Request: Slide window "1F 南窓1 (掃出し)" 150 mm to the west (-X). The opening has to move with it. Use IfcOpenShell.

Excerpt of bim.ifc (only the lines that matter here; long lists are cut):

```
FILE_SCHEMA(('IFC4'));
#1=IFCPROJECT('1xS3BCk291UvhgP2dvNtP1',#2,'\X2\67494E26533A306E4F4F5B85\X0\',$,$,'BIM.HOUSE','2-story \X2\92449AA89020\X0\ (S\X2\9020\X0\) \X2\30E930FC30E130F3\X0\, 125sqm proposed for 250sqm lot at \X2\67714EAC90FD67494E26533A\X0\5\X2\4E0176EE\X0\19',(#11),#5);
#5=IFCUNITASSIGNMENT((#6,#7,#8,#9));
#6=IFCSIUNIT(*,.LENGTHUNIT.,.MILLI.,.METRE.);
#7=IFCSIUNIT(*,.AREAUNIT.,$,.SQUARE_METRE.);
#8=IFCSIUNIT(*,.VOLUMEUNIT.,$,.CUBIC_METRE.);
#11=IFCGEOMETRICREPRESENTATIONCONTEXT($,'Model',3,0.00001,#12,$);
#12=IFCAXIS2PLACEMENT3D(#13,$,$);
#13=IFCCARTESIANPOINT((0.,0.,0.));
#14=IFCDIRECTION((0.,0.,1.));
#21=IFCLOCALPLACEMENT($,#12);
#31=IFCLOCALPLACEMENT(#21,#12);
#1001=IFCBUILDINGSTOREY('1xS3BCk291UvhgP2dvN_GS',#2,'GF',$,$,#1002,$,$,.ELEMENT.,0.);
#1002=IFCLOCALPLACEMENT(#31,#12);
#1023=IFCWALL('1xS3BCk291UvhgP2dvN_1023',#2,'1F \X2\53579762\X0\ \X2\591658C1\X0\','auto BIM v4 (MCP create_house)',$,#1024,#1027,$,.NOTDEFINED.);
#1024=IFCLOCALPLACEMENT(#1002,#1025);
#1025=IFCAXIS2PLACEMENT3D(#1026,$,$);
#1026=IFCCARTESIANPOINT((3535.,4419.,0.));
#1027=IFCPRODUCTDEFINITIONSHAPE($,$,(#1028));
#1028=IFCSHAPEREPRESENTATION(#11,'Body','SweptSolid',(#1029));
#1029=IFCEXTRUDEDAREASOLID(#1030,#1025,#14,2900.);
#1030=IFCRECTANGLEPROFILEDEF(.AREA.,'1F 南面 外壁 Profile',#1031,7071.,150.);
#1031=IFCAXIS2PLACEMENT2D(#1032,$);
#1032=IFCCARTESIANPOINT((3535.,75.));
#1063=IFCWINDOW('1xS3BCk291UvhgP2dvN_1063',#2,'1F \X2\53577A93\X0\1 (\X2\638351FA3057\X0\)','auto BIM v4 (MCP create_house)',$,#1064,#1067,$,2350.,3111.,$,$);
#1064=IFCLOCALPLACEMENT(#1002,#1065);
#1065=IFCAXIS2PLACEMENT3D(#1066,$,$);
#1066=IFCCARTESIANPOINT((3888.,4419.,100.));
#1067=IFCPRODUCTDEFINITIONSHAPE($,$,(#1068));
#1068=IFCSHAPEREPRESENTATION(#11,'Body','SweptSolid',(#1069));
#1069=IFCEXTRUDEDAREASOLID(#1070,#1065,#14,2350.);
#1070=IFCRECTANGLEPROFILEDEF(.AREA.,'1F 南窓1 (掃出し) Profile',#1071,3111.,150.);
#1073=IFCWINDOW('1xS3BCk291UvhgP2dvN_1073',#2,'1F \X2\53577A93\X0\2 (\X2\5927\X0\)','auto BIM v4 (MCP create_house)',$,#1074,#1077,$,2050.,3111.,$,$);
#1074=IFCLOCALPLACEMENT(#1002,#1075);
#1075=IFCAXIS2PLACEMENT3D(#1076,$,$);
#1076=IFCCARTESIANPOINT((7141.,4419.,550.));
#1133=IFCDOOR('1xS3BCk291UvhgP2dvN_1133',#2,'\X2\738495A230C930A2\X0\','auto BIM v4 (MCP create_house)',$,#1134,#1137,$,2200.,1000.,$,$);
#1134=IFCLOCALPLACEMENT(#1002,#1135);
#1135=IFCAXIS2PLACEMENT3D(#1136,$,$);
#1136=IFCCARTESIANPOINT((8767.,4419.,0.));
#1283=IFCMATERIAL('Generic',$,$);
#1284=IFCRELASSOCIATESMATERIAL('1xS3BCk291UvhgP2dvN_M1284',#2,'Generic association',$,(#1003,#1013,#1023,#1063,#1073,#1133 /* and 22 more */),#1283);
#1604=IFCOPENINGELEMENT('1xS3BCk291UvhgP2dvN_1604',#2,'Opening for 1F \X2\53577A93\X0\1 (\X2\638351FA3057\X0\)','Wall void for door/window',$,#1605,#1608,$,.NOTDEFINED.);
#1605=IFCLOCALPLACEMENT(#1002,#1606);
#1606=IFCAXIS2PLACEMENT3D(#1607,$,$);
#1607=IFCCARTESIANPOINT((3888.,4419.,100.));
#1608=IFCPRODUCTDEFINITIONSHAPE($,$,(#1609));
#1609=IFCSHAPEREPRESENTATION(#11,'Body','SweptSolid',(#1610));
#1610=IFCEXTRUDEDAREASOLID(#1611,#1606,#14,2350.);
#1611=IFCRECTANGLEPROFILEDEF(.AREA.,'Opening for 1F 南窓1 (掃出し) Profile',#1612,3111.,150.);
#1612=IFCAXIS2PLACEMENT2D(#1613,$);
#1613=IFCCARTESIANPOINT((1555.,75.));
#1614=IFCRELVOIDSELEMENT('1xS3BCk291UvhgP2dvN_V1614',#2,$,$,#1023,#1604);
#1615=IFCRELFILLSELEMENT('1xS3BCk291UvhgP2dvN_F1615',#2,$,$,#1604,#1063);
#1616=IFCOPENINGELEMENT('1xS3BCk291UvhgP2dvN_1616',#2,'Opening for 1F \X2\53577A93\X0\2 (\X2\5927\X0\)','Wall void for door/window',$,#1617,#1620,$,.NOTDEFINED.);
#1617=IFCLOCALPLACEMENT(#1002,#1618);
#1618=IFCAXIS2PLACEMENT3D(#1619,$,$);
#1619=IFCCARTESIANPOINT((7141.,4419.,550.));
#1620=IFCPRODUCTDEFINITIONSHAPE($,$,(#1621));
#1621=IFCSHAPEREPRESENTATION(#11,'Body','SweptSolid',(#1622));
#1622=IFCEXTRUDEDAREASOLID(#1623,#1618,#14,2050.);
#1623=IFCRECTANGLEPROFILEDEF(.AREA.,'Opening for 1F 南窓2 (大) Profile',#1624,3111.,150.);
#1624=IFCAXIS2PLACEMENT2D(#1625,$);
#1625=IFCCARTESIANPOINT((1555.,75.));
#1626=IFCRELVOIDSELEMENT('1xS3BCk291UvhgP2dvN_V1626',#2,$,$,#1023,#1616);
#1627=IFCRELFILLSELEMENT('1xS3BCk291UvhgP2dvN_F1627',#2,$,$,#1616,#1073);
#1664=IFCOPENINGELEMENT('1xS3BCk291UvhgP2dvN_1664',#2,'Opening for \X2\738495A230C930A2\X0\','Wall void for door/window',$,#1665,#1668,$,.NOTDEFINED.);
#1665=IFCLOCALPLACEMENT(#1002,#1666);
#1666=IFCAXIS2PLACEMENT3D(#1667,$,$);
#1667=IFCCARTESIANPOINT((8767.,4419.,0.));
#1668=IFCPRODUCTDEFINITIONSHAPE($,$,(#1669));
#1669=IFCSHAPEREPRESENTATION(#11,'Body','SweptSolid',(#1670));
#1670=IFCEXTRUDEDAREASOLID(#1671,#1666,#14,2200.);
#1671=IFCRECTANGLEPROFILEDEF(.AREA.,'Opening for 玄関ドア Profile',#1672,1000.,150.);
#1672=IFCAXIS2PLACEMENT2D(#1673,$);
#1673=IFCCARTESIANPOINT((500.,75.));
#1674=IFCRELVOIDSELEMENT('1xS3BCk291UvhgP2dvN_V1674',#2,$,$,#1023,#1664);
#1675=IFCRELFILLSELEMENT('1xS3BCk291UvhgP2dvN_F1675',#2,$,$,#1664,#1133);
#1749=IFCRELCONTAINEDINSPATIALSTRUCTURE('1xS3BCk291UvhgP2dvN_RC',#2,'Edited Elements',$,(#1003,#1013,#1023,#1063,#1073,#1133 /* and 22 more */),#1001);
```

```python
import ifcopenshell
import ifcopenshell.api.geometry
import ifcopenshell.util.placement
import ifcopenshell.util.unit

model = ifcopenshell.open("bim.ifc")
unit_scale = ifcopenshell.util.unit.calculate_unit_scale(model)

window = model.by_guid("1xS3BCk291UvhgP2dvN_1063")
opening = window.FillsVoids[0].RelatingOpeningElement
wall = opening.VoidsElements[0].RelatingBuildingElement

wall_matrix = ifcopenshell.util.placement.get_local_placement(wall.ObjectPlacement)
shift = wall_matrix[:3, 0] * -0.15 / unit_scale
before = ifcopenshell.util.placement.get_local_placement(window.ObjectPlacement)[:3, 3].copy()

# The window is not placed relative to its opening, so move both.
for product in (opening, window):
    matrix = ifcopenshell.util.placement.get_local_placement(product.ObjectPlacement)
    matrix[:3, 3] += shift
    ifcopenshell.api.geometry.edit_object_placement(model, product=product, matrix=matrix, is_si=False)

after = ifcopenshell.util.placement.get_local_placement(window.ObjectPlacement)[:3, 3]
print("window moved by", (after - before).round(3) + 0.0)

model.write("bim_updated.ifc")
```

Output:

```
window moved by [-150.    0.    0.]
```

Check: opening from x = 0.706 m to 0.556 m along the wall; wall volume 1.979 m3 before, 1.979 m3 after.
